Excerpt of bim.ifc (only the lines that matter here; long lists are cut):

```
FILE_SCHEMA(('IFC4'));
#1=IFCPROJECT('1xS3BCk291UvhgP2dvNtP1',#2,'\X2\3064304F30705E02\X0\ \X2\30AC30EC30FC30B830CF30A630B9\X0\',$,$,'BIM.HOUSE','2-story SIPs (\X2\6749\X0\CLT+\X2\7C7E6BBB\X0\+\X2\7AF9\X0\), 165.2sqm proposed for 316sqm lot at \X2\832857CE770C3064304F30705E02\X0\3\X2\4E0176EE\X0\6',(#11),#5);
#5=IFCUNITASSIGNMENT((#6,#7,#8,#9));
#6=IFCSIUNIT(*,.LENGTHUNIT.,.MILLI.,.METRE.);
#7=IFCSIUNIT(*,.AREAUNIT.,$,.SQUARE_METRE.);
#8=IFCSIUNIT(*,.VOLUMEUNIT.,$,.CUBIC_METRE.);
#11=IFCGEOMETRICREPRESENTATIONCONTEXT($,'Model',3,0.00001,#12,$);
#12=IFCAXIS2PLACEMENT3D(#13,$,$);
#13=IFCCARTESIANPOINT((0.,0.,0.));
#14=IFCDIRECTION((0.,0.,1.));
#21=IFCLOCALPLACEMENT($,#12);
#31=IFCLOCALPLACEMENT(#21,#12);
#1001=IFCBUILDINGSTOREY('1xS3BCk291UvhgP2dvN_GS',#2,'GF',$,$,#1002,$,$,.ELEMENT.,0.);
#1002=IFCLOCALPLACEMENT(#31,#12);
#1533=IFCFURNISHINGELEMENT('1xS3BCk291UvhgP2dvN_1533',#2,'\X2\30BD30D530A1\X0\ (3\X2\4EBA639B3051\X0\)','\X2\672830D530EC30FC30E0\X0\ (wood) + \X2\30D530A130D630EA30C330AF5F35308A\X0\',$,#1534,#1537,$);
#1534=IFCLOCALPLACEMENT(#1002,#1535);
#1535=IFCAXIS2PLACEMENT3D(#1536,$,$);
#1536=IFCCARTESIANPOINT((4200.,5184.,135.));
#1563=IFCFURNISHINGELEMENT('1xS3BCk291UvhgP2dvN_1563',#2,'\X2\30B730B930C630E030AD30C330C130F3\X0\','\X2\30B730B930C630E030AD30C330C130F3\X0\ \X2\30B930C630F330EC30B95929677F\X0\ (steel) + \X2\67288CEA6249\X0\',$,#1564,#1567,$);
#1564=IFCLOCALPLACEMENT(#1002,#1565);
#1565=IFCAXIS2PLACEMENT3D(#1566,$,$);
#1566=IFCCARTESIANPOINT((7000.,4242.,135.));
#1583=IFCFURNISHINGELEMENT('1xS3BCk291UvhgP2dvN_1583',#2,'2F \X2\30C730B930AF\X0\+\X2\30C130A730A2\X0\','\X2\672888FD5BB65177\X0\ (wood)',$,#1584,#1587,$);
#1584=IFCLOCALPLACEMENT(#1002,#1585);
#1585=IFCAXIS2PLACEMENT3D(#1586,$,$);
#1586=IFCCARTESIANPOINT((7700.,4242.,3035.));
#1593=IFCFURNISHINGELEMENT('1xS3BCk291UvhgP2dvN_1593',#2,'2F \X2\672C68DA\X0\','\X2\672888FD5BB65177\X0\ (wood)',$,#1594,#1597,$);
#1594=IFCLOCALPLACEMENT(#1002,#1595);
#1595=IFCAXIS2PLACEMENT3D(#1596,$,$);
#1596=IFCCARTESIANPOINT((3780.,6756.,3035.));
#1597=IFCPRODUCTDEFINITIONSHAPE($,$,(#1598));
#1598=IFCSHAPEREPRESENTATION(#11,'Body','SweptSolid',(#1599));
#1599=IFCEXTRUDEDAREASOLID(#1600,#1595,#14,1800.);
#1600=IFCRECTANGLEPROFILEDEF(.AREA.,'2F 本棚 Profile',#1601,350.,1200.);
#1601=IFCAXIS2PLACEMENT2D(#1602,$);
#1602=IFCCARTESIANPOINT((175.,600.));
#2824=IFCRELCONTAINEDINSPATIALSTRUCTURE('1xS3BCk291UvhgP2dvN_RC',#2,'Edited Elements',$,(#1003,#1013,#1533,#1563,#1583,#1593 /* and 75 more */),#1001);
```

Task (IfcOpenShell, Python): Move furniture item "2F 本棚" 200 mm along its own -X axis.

```python
import ifcopenshell
import ifcopenshell.api.geometry
import ifcopenshell.util.placement

model = ifcopenshell.open("bim.ifc")

item = model.by_guid("1xS3BCk291UvhgP2dvN_1593")
matrix = ifcopenshell.util.placement.get_local_placement(item.ObjectPlacement)
matrix[:3, 3] -= matrix[:3, 0] * 200.0
ifcopenshell.api.geometry.edit_object_placement(model, product=item, matrix=matrix, is_si=False)

print(ifcopenshell.util.placement.get_local_placement(item.ObjectPlacement).round(3) + 0.0)

model.write("bim_v2.ifc")
```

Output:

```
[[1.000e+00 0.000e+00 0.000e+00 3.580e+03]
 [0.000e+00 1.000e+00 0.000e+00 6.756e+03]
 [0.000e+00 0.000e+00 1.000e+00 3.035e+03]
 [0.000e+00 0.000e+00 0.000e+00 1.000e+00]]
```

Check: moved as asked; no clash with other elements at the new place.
